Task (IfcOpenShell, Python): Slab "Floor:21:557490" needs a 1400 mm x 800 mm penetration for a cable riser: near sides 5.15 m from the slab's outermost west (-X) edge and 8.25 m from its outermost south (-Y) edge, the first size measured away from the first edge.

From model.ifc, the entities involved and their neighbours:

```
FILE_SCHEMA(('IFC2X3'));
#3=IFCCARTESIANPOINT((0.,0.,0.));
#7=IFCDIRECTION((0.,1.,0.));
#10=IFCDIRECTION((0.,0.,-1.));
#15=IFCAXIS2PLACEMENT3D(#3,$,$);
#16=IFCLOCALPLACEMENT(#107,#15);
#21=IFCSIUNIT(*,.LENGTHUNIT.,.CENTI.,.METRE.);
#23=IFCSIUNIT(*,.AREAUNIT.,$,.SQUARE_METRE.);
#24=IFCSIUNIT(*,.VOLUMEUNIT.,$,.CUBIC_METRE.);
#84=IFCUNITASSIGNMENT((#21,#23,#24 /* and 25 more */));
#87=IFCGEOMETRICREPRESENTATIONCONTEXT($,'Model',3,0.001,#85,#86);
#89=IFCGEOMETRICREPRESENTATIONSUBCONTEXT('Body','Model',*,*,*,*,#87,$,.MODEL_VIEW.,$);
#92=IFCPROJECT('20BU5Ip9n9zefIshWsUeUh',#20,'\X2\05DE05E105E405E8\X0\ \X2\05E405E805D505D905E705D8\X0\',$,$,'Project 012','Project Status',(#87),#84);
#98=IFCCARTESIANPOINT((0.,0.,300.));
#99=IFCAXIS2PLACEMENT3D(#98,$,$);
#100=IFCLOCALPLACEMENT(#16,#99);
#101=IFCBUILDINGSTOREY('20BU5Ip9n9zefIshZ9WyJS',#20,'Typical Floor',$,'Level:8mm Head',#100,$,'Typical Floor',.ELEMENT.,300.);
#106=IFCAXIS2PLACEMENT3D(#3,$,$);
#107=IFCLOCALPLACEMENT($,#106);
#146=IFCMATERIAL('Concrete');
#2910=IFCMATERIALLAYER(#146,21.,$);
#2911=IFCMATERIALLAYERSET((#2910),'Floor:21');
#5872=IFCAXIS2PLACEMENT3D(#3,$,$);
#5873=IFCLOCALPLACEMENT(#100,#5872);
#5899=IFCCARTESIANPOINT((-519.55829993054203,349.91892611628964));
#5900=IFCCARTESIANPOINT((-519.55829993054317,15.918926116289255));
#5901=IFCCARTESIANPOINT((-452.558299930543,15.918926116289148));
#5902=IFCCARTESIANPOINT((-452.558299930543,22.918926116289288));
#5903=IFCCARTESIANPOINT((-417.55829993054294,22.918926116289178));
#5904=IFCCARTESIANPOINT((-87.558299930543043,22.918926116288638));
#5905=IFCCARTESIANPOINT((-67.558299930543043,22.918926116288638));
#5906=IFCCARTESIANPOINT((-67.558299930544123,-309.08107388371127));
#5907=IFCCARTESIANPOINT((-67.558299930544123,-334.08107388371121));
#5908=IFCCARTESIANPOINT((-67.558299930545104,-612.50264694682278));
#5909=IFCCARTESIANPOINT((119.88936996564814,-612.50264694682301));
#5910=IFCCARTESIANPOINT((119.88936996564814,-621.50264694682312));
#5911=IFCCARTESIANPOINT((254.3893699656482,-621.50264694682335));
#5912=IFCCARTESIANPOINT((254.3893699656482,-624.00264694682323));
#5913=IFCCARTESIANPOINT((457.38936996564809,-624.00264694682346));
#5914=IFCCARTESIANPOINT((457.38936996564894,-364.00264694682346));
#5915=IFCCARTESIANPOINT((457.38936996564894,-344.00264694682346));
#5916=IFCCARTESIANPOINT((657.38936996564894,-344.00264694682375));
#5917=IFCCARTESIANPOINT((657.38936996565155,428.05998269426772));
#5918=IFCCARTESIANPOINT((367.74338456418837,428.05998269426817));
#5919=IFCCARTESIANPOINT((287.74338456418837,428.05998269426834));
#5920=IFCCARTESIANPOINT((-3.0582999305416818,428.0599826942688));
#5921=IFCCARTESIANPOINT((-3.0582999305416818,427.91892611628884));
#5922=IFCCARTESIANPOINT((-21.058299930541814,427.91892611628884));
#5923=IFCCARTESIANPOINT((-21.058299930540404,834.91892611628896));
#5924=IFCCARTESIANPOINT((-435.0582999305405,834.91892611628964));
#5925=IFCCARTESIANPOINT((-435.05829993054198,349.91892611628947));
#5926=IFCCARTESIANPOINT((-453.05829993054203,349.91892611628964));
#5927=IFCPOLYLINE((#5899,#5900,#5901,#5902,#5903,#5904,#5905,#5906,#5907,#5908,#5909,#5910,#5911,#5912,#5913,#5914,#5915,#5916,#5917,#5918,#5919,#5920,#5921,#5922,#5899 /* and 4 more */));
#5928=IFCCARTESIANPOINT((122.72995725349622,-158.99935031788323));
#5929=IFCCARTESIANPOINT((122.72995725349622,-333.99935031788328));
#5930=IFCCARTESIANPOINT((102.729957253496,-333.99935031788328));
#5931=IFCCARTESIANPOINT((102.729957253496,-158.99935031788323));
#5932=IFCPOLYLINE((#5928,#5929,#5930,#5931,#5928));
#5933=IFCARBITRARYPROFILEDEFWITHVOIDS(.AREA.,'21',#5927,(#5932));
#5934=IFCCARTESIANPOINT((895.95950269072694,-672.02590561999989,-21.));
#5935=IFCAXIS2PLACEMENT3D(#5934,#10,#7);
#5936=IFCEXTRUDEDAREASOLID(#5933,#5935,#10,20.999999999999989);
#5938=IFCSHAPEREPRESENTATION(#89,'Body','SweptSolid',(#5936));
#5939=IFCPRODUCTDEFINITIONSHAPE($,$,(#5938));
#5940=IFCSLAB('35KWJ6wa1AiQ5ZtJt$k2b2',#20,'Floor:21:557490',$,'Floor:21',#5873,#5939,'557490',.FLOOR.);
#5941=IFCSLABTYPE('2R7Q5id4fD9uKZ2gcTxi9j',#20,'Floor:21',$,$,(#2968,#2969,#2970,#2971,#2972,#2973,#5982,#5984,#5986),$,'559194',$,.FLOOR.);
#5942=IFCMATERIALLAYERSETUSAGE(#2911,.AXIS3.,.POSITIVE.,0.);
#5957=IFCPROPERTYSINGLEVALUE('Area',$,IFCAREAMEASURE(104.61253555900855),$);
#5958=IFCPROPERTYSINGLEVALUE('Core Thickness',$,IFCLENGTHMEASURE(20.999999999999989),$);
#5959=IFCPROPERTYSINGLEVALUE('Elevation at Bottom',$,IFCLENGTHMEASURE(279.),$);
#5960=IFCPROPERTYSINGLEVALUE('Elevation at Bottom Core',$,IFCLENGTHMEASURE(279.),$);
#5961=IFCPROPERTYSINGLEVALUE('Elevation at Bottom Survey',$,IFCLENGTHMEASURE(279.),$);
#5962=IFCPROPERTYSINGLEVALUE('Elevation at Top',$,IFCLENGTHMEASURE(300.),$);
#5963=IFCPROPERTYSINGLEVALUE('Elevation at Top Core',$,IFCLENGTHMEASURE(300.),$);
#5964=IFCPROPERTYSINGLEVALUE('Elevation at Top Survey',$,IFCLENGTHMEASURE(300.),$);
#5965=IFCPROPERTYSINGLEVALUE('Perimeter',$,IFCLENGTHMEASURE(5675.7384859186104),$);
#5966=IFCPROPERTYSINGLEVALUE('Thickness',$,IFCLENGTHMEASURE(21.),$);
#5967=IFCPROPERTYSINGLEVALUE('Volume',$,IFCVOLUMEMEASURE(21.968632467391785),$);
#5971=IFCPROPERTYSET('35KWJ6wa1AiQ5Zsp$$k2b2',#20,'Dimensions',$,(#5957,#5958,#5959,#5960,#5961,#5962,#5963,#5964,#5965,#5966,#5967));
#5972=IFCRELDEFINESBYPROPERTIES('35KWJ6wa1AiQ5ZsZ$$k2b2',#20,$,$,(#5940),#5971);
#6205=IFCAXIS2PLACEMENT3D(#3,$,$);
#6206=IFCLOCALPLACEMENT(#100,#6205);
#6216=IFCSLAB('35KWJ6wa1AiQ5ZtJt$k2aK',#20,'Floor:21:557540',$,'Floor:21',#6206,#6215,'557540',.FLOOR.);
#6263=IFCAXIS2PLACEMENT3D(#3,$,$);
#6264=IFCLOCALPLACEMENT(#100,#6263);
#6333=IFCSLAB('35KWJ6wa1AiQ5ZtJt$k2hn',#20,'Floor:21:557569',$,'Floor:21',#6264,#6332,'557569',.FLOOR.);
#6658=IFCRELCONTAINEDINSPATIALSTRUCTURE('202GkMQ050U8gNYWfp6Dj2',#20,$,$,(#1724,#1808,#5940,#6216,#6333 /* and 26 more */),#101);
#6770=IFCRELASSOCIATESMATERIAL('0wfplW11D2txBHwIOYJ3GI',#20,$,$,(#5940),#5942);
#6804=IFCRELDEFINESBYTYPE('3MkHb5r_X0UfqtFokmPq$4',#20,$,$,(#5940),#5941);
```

```python
import numpy as np
import ifcopenshell
import ifcopenshell.api.feature
import ifcopenshell.api.geometry
import ifcopenshell.api.pset
import ifcopenshell.api.root
import ifcopenshell.geom
import ifcopenshell.util.element
import ifcopenshell.util.placement
import ifcopenshell.util.representation
import ifcopenshell.util.shape
import ifcopenshell.util.unit

model = ifcopenshell.open("model.ifc")
unit_scale = ifcopenshell.util.unit.calculate_unit_scale(model)
area_scale = ifcopenshell.util.unit.calculate_unit_scale(model, "AREAUNIT")
volume_scale = ifcopenshell.util.unit.calculate_unit_scale(model, "VOLUMEUNIT")
settings = ifcopenshell.geom.settings()


def volume(element):
    """Net volume in cubic metres, openings subtracted."""
    shape = ifcopenshell.geom.create_shape(settings, element)
    return ifcopenshell.util.shape.get_volume(shape.geometry)


slab = model.by_guid("35KWJ6wa1AiQ5ZtJt$k2b2")
before = volume(slab)

# Extent in the slab's own axes, in metres. The edges named are its -X and -Y sides.
slab_shape = ifcopenshell.geom.create_shape(settings, slab)
vertices = ifcopenshell.util.shape.get_vertices(slab_shape.geometry)
x_min, y_min, bottom = vertices.min(axis=0)
top = vertices[:, 2].max()

opening = ifcopenshell.api.root.create_entity(model, ifc_class="IfcOpeningElement", name="Cable riser opening")
context = ifcopenshell.util.representation.get_context(model, "Model", "Body", "MODEL_VIEW")
width, depth = 1.4, 0.8
outline = [(0.0, 0.0), (width, 0.0), (width, depth), (0.0, depth), (0.0, 0.0)]
# Overshoot both faces by 50 mm so the cut is clean.
shape = ifcopenshell.api.geometry.add_slab_representation(
    model, context=context, depth=top - bottom + 0.1, polyline=outline
)
ifcopenshell.api.geometry.assign_representation(model, product=opening, representation=shape)

matrix = ifcopenshell.util.placement.get_local_placement(slab.ObjectPlacement)
matrix[:, 3] = matrix @ np.append(np.array([x_min + 5.15, y_min + 8.25, bottom - 0.05]) / unit_scale, 1.0)
ifcopenshell.api.geometry.edit_object_placement(model, product=opening, matrix=matrix, is_si=False)
ifcopenshell.api.feature.add_feature(model, feature=opening, element=slab)

after = volume(slab)

# Update the slab's stored quantities.
pset = model.by_id(ifcopenshell.util.element.get_pset(slab, "Dimensions", should_inherit=False)["id"])
ifcopenshell.api.pset.edit_pset(model, pset=pset, properties={
    "Area": model.create_entity("IfcAreaMeasure", after / (top - bottom) / area_scale),
    "Volume": model.create_entity("IfcVolumeMeasure", after / volume_scale),
})

print(f"slab volume {before:.3f} -> {after:.3f} m3")

model.write("model_updated.ifc")
```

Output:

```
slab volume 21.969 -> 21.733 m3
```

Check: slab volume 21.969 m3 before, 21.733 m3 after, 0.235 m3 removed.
